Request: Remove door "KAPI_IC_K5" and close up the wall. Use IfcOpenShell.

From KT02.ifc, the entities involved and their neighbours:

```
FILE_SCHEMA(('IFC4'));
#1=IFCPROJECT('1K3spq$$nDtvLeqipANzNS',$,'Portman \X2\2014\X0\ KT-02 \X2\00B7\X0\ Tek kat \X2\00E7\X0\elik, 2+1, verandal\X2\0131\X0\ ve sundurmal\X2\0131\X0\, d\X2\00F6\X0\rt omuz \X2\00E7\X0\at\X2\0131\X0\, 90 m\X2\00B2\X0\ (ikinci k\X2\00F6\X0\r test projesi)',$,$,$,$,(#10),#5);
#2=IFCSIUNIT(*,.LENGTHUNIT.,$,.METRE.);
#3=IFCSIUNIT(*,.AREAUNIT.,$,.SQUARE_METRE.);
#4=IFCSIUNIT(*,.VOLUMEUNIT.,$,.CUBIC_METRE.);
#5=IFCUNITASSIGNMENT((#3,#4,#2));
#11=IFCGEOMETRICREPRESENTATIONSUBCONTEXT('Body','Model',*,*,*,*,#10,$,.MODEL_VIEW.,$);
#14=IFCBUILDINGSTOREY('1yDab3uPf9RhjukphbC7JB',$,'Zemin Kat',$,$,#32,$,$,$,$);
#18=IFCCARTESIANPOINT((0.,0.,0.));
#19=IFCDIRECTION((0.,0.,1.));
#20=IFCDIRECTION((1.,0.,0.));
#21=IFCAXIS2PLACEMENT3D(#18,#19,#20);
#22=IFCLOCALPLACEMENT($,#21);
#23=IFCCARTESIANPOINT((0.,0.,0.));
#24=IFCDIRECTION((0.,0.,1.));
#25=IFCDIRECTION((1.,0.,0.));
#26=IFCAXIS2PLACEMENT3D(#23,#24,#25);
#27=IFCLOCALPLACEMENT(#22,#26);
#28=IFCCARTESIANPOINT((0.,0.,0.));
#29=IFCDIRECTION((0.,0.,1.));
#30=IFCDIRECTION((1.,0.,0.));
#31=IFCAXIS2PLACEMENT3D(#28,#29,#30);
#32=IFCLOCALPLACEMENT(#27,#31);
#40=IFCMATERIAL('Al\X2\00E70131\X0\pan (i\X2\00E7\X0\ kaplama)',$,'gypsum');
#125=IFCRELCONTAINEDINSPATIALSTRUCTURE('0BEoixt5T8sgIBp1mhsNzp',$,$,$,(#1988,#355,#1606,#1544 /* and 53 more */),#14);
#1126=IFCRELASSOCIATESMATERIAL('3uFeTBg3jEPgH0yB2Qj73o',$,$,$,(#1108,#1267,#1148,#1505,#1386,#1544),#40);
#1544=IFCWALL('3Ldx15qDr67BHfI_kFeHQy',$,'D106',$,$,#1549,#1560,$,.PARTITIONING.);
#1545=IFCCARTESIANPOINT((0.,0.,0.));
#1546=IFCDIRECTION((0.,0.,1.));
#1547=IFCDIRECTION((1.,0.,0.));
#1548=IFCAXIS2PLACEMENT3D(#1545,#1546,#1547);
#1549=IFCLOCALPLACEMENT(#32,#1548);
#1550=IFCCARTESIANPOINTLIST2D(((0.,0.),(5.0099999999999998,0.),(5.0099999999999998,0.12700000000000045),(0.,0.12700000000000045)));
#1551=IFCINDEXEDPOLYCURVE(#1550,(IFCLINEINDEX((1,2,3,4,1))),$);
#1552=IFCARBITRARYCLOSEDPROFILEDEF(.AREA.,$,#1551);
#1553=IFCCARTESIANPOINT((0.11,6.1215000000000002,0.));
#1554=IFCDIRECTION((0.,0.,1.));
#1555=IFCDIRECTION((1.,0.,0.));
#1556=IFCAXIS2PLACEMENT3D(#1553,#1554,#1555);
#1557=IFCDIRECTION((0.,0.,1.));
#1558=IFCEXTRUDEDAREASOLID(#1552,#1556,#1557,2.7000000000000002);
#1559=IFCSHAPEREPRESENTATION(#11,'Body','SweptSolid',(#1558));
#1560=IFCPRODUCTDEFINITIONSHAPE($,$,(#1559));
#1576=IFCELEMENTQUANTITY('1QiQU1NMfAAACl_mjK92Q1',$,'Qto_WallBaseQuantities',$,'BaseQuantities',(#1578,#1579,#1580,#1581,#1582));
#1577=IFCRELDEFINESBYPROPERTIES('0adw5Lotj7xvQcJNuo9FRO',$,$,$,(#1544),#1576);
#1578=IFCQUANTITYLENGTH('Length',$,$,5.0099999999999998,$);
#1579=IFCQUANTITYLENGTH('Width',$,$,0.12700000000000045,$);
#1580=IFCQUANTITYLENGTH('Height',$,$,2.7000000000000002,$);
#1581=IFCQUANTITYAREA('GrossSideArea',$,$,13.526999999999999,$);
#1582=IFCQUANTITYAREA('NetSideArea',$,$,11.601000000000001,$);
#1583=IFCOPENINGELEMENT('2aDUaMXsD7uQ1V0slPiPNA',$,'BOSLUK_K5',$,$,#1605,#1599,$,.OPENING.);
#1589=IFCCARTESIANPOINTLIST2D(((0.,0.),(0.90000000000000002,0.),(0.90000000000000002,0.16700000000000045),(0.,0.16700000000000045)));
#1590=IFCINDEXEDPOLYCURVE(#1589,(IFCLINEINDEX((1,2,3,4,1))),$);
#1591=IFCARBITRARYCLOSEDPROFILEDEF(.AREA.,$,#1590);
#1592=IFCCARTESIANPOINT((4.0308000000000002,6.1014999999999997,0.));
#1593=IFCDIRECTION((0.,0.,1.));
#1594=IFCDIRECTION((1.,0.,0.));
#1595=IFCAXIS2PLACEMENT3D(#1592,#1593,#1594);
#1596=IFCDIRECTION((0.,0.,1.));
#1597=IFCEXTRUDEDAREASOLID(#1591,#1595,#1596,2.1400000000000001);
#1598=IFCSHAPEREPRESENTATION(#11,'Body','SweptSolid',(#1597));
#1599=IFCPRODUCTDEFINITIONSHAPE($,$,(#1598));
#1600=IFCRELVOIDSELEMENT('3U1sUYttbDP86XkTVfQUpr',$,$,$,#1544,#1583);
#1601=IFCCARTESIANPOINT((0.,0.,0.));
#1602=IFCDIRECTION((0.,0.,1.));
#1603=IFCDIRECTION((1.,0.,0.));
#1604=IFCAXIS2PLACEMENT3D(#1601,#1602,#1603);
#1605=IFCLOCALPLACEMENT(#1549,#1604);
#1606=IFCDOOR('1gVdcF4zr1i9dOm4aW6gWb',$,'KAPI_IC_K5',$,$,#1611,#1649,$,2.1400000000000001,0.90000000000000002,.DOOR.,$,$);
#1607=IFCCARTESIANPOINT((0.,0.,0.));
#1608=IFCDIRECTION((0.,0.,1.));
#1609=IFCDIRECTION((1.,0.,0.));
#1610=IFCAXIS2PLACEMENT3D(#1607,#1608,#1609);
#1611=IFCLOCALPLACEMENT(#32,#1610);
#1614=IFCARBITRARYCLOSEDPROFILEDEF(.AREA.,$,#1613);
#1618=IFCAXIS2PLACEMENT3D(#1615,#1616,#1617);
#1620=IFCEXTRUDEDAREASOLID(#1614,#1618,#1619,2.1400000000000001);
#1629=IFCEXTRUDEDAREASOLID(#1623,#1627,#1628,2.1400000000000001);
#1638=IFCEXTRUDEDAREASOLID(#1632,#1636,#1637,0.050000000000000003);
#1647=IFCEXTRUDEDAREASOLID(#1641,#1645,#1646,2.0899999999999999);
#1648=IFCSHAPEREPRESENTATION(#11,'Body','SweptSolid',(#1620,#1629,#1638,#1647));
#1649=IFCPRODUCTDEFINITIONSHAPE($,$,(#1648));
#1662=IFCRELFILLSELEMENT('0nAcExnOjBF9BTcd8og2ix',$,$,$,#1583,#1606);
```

```python
import ifcopenshell
import ifcopenshell.api.feature
import ifcopenshell.api.pset
import ifcopenshell.api.root
import ifcopenshell.geom
import ifcopenshell.util.element
import ifcopenshell.util.shape
import ifcopenshell.util.unit

model = ifcopenshell.open("KT02.ifc")
area_scale = ifcopenshell.util.unit.calculate_unit_scale(model, "AREAUNIT")
settings = ifcopenshell.geom.settings()


def volume(element):
    """Net volume in cubic metres, openings subtracted."""
    shape = ifcopenshell.geom.create_shape(settings, element)
    return ifcopenshell.util.shape.get_volume(shape.geometry)


door = model.by_guid("1gVdcF4zr1i9dOm4aW6gWb")
opening = door.FillsVoids[0].RelatingOpeningElement
wall = opening.VoidsElements[0].RelatingBuildingElement
before = volume(wall)

ifcopenshell.api.root.remove_product(model, product=door)
ifcopenshell.api.feature.remove_feature(model, feature=opening)

after = volume(wall)
thickness = 0.127  # wall thickness in metres

# Update the wall's stored quantities.
qto = model.by_id(ifcopenshell.util.element.get_pset(wall, "Qto_WallBaseQuantities", should_inherit=False)["id"])
ifcopenshell.api.pset.edit_qto(model, qto=qto, properties={"NetSideArea": after / thickness / area_scale})

print(f"wall volume {before:.3f} -> {after:.3f} m3")

model.write("KT02_updated.ifc")
```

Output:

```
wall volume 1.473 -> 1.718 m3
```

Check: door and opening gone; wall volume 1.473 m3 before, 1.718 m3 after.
